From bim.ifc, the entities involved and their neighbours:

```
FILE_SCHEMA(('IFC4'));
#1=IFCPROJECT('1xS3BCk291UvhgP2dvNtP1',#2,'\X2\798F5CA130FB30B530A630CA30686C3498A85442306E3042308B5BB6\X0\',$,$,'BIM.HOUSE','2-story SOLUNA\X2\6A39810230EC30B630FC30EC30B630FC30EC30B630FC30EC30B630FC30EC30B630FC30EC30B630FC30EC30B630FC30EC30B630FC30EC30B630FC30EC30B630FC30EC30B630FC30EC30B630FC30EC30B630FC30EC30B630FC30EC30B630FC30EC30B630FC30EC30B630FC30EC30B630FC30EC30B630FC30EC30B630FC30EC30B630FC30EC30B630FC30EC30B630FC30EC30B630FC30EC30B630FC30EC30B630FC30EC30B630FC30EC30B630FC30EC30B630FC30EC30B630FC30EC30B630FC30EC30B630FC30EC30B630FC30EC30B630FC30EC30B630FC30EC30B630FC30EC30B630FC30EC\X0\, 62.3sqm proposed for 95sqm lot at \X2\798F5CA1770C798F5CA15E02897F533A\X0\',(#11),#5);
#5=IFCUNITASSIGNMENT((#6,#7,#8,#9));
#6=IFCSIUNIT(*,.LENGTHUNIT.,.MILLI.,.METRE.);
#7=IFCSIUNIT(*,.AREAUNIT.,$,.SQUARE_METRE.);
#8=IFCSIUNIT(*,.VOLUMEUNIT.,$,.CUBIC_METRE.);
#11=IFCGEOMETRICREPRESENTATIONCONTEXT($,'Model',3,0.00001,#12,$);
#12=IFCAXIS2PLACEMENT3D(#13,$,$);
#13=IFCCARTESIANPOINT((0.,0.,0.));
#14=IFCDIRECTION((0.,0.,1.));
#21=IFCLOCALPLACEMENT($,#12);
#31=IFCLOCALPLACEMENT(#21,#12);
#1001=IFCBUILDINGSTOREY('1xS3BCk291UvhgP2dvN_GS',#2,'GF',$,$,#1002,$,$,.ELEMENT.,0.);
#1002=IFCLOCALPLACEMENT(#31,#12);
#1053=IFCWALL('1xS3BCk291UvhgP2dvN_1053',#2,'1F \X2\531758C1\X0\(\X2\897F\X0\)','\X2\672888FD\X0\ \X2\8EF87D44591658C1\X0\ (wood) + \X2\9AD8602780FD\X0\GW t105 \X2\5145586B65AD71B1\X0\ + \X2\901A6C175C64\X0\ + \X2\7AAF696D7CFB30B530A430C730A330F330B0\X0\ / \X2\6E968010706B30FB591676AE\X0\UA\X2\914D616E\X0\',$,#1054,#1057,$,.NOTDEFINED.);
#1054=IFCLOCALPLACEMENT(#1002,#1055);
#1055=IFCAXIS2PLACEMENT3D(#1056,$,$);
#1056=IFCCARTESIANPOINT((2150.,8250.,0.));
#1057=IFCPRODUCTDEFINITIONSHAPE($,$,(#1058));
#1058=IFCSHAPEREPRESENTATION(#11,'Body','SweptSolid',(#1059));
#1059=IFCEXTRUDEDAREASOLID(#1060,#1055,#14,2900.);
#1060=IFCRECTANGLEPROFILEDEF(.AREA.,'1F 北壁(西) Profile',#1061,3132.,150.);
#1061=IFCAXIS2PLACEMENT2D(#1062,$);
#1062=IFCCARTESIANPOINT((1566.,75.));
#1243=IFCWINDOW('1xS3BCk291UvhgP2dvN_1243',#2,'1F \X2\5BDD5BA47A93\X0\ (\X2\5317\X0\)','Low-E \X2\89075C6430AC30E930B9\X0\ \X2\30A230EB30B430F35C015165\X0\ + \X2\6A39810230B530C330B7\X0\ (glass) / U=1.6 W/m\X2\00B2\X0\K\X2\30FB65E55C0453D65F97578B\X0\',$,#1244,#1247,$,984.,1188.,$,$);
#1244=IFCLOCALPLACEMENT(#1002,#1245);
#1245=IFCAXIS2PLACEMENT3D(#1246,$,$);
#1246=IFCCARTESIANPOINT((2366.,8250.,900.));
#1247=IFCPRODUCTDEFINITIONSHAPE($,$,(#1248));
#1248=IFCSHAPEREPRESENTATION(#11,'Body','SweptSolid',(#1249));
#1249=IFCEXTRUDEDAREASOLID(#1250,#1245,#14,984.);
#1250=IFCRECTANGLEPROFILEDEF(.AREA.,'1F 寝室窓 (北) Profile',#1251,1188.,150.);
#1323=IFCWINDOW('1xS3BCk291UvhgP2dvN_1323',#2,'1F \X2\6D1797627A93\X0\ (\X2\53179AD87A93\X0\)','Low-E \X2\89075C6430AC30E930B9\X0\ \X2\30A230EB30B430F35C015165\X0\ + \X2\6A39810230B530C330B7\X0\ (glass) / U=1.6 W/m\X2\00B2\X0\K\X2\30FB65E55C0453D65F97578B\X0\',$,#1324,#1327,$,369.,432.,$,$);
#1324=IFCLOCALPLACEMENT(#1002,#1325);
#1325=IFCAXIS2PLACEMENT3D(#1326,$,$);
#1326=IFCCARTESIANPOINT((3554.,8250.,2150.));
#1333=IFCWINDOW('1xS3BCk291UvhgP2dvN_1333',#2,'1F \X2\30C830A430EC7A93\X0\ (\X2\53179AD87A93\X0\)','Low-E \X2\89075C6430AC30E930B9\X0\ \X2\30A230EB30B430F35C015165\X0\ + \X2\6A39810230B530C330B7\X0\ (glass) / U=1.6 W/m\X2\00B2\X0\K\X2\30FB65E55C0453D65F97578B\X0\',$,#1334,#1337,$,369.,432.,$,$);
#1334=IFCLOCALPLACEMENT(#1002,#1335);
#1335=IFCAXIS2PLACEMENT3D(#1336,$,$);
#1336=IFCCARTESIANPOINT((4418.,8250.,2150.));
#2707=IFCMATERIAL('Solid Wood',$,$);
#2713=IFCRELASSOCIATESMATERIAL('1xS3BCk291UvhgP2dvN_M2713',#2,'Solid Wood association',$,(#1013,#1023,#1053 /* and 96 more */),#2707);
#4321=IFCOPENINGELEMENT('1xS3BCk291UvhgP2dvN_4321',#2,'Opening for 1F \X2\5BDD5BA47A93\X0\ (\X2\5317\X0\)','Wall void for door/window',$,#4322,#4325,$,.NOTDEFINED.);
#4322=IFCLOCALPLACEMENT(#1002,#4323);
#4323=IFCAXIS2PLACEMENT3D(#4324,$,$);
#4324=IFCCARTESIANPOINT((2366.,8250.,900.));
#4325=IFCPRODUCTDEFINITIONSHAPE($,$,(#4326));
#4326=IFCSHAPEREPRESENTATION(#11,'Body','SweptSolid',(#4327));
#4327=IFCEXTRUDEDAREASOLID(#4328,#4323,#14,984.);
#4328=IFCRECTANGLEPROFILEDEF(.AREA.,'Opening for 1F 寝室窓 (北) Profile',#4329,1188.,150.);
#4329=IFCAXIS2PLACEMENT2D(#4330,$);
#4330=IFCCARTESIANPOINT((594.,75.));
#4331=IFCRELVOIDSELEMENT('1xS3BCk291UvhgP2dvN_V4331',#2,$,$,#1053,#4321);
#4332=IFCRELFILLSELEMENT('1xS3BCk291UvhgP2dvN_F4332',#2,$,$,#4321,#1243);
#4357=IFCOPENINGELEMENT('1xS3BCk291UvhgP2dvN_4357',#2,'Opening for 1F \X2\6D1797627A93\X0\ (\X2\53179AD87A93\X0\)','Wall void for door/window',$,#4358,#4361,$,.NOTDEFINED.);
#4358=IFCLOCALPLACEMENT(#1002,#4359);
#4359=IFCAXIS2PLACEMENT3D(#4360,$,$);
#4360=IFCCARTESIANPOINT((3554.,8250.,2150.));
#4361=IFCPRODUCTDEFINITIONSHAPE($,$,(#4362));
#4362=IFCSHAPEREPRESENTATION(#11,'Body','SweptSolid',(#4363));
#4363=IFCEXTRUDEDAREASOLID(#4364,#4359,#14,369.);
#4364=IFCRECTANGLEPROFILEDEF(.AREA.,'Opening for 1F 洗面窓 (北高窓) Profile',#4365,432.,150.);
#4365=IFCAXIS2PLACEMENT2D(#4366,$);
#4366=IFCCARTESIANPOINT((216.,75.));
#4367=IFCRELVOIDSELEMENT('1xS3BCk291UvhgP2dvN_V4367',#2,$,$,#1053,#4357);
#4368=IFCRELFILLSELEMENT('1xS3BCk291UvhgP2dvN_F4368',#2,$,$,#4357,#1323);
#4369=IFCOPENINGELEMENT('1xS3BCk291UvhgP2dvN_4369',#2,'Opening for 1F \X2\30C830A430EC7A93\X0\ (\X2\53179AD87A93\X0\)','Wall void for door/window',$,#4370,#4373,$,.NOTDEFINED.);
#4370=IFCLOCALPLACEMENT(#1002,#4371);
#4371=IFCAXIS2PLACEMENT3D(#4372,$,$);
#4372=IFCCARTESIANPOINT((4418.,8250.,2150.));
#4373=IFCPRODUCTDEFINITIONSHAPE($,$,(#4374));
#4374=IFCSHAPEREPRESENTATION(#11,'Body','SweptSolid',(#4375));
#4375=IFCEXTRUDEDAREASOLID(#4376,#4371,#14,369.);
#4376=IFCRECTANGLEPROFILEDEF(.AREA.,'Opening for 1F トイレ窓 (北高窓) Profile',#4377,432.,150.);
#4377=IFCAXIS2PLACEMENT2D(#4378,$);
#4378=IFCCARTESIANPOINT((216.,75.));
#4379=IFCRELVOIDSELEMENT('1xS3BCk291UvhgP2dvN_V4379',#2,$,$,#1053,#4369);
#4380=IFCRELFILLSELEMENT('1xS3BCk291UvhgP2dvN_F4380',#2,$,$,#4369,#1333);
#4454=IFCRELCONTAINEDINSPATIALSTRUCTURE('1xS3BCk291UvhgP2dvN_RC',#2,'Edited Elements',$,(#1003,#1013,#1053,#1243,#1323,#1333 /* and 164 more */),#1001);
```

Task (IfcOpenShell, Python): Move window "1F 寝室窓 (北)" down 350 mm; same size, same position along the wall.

```python
import numpy as np
import ifcopenshell
import ifcopenshell.api.geometry
import ifcopenshell.util.placement
import ifcopenshell.util.unit

model = ifcopenshell.open("bim.ifc")
unit_scale = ifcopenshell.util.unit.calculate_unit_scale(model)

window = model.by_guid("1xS3BCk291UvhgP2dvN_1243")
opening = window.FillsVoids[0].RelatingOpeningElement
dz = -350.0

shift = np.array([0.0, 0.0, dz])
# The window is not placed relative to its opening, so move both.
for product in (opening, window):
    matrix = ifcopenshell.util.placement.get_local_placement(product.ObjectPlacement)
    matrix[:3, 3] += shift
    ifcopenshell.api.geometry.edit_object_placement(model, product=product, matrix=matrix, is_si=False)

print(f"moved by {dz * unit_scale:+.3f} m")

model.write("bim_v2.ifc")
```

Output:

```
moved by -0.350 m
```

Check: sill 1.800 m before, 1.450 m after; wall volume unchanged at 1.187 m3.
